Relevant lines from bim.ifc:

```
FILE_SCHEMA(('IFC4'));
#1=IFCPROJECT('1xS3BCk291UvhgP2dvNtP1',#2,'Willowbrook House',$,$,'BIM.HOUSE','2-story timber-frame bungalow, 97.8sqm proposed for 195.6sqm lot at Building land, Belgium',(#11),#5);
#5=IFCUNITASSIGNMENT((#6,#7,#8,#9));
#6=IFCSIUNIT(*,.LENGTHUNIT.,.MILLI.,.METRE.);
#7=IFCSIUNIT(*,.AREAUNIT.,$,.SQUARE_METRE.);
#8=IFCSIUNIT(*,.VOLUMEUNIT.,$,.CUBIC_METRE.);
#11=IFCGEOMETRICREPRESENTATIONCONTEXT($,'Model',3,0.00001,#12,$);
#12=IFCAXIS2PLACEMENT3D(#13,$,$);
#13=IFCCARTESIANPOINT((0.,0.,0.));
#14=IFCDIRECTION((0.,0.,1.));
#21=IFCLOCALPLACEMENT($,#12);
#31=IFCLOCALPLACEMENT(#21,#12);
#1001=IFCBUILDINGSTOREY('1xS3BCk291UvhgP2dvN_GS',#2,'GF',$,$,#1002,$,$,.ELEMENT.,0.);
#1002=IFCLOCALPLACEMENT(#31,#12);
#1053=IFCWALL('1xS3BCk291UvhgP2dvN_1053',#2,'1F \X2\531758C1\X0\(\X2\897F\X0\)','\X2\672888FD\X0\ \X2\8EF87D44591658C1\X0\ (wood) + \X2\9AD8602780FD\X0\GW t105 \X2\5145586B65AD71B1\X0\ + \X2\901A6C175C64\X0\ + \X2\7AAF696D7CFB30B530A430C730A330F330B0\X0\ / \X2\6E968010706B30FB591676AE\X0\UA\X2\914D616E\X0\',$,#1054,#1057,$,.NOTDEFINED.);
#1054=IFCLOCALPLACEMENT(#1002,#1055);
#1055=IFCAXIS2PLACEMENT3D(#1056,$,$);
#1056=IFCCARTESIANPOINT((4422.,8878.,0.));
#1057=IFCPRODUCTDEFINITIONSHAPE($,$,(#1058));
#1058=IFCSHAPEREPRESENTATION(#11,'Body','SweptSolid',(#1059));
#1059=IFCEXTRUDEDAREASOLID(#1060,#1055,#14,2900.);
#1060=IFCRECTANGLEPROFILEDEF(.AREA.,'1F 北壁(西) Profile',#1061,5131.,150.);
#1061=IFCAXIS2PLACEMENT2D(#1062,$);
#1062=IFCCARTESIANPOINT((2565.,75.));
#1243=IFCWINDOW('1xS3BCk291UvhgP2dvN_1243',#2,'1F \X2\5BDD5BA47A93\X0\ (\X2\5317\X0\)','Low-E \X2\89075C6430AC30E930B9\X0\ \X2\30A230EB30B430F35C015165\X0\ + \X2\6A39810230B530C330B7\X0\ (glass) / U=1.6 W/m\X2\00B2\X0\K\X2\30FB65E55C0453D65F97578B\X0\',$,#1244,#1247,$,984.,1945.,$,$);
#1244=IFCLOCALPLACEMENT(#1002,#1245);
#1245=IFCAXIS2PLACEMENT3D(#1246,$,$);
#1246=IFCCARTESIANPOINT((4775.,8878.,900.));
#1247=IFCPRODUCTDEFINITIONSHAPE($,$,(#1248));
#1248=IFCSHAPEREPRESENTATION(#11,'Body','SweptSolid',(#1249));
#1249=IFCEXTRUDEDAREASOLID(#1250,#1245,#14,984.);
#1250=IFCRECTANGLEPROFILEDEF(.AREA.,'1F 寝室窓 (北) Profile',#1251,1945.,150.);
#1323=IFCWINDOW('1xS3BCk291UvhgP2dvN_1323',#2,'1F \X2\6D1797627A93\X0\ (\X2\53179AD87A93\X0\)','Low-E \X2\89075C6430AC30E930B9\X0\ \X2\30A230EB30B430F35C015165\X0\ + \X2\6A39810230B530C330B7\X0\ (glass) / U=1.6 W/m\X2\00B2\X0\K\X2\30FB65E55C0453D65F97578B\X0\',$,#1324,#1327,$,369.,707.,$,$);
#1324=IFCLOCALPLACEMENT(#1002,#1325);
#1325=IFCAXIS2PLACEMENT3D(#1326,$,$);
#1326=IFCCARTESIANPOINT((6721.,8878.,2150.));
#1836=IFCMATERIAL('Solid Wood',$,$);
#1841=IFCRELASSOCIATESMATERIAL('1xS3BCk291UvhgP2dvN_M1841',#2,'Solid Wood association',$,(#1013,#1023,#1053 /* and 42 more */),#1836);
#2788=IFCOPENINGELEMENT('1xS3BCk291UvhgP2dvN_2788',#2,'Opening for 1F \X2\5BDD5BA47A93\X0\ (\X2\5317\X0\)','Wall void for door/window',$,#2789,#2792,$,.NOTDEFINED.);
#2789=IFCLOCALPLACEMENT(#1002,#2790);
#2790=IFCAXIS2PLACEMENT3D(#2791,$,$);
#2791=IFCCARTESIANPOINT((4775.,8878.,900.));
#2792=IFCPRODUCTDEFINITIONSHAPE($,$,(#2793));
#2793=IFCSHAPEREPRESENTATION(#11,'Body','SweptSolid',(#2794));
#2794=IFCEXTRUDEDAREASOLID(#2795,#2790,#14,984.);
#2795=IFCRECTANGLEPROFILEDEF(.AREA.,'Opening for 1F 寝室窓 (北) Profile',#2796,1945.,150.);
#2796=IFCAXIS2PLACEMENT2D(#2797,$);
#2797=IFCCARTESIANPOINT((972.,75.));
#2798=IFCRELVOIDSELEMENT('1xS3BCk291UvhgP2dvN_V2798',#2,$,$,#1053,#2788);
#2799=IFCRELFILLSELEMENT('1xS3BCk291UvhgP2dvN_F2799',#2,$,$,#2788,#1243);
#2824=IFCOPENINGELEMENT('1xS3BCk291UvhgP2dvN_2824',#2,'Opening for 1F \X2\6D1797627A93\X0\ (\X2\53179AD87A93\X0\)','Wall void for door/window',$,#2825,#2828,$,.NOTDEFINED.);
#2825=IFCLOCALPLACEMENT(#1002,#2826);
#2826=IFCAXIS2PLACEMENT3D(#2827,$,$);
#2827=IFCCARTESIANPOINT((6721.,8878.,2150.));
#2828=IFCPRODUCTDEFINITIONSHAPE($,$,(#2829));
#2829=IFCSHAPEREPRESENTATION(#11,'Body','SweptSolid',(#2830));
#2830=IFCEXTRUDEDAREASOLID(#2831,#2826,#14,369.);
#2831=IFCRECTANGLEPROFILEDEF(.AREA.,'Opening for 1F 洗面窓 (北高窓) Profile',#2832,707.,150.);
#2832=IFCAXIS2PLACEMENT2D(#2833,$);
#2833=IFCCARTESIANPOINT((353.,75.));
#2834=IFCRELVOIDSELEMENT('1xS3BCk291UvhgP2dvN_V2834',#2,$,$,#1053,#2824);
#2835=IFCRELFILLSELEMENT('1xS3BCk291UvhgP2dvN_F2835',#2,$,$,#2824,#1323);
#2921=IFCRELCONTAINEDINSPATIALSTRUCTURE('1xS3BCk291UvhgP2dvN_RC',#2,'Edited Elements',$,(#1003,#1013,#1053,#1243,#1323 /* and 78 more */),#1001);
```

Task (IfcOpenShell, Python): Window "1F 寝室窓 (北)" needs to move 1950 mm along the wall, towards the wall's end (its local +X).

```python
import ifcopenshell
import ifcopenshell.api.geometry
import ifcopenshell.util.placement

model = ifcopenshell.open("bim.ifc")

window = model.by_id(1243)
opening = window.FillsVoids[0].RelatingOpeningElement
wall = opening.VoidsElements[0].RelatingBuildingElement

wall_matrix = ifcopenshell.util.placement.get_local_placement(wall.ObjectPlacement)
shift = wall_matrix[:3, 0] * 1950.0
before = ifcopenshell.util.placement.get_local_placement(window.ObjectPlacement)[:3, 3].copy()

# The window is not placed relative to its opening, so move both.
for product in (opening, window):
    matrix = ifcopenshell.util.placement.get_local_placement(product.ObjectPlacement)
    matrix[:3, 3] += shift
    ifcopenshell.api.geometry.edit_object_placement(model, product=product, matrix=matrix, is_si=False)

after = ifcopenshell.util.placement.get_local_placement(window.ObjectPlacement)[:3, 3]
print("window moved by", (after - before).round(3) + 0.0)

model.write("bim-out.ifc")
```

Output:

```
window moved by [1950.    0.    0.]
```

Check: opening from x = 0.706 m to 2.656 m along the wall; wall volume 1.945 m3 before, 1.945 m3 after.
